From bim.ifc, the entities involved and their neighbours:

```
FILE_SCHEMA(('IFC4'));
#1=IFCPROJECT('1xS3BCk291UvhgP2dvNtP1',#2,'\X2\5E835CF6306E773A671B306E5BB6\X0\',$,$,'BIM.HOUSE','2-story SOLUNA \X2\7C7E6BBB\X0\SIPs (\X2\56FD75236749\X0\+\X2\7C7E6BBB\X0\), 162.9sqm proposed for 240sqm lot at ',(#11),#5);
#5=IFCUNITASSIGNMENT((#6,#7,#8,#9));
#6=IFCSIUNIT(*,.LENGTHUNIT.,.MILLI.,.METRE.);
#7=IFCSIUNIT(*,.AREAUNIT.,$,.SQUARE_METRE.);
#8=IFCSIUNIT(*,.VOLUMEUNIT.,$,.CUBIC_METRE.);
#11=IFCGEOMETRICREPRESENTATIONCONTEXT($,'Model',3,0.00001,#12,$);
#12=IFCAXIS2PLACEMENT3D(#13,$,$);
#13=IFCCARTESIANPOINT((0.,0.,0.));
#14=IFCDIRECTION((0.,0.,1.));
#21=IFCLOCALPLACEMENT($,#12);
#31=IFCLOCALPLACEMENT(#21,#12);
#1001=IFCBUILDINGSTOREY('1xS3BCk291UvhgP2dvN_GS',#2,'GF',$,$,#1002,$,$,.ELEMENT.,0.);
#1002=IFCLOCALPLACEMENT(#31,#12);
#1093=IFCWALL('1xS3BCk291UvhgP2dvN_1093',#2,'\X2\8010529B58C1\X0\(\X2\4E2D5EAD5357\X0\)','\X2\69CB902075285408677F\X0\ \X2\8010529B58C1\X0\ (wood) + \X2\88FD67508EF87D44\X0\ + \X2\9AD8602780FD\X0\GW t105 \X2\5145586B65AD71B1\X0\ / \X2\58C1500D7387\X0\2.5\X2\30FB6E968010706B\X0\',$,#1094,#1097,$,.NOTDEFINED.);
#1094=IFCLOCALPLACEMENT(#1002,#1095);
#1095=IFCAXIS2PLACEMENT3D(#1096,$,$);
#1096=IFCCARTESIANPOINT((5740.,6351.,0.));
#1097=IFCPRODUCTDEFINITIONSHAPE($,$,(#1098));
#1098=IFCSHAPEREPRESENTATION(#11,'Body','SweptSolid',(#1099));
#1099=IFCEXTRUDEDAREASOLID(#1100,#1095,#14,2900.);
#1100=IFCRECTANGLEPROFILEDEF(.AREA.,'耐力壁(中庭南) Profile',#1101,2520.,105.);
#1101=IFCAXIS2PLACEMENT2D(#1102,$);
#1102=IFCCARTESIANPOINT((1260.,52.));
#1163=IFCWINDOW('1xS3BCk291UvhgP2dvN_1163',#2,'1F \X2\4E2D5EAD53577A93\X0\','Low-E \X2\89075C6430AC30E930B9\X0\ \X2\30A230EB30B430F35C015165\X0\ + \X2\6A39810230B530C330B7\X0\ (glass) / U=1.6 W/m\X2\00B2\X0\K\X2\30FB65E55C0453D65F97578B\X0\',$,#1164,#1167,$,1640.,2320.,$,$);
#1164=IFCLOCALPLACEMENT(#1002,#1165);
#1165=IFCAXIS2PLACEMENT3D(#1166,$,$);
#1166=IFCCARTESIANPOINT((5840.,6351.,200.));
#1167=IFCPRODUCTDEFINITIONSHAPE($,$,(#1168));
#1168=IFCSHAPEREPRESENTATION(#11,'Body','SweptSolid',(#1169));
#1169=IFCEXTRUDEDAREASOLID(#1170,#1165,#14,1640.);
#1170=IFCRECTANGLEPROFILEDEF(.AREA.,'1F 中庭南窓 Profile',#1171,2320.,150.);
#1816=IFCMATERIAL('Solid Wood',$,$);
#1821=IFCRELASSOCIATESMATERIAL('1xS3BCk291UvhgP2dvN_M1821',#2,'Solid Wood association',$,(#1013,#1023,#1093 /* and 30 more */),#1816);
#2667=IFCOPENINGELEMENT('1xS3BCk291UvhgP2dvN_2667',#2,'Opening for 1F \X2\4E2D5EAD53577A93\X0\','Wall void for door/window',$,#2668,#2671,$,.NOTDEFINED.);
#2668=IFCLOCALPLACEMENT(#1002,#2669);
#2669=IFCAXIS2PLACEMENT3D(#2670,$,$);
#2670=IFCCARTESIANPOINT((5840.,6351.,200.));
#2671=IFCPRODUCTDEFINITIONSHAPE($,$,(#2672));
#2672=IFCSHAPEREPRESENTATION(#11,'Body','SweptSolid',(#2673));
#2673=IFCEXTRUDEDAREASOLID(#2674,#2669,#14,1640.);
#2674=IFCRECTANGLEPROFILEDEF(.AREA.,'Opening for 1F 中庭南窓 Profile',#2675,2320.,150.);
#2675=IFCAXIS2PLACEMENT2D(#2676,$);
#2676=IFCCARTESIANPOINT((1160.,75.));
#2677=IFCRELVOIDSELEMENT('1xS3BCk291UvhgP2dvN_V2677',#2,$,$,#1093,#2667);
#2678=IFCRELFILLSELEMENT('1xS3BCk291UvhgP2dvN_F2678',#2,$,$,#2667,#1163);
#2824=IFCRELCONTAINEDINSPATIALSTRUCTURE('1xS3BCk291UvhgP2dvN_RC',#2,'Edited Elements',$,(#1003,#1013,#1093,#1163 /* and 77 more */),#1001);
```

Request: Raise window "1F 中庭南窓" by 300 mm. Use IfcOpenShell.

```python
import numpy as np
import ifcopenshell
import ifcopenshell.api.geometry
import ifcopenshell.util.placement
import ifcopenshell.util.unit

model = ifcopenshell.open("bim.ifc")
unit_scale = ifcopenshell.util.unit.calculate_unit_scale(model)

window = model.by_id(1163)
opening = window.FillsVoids[0].RelatingOpeningElement
dz = 0.3 / unit_scale

shift = np.array([0.0, 0.0, dz])
# The window is not placed relative to its opening, so move both.
for product in (opening, window):
    matrix = ifcopenshell.util.placement.get_local_placement(product.ObjectPlacement)
    matrix[:3, 3] += shift
    ifcopenshell.api.geometry.edit_object_placement(model, product=product, matrix=matrix, is_si=False)

print(f"moved by {dz * unit_scale:+.3f} m")

model.write("bim_rev.ifc")
```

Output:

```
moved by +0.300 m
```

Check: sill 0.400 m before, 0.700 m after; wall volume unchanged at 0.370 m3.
